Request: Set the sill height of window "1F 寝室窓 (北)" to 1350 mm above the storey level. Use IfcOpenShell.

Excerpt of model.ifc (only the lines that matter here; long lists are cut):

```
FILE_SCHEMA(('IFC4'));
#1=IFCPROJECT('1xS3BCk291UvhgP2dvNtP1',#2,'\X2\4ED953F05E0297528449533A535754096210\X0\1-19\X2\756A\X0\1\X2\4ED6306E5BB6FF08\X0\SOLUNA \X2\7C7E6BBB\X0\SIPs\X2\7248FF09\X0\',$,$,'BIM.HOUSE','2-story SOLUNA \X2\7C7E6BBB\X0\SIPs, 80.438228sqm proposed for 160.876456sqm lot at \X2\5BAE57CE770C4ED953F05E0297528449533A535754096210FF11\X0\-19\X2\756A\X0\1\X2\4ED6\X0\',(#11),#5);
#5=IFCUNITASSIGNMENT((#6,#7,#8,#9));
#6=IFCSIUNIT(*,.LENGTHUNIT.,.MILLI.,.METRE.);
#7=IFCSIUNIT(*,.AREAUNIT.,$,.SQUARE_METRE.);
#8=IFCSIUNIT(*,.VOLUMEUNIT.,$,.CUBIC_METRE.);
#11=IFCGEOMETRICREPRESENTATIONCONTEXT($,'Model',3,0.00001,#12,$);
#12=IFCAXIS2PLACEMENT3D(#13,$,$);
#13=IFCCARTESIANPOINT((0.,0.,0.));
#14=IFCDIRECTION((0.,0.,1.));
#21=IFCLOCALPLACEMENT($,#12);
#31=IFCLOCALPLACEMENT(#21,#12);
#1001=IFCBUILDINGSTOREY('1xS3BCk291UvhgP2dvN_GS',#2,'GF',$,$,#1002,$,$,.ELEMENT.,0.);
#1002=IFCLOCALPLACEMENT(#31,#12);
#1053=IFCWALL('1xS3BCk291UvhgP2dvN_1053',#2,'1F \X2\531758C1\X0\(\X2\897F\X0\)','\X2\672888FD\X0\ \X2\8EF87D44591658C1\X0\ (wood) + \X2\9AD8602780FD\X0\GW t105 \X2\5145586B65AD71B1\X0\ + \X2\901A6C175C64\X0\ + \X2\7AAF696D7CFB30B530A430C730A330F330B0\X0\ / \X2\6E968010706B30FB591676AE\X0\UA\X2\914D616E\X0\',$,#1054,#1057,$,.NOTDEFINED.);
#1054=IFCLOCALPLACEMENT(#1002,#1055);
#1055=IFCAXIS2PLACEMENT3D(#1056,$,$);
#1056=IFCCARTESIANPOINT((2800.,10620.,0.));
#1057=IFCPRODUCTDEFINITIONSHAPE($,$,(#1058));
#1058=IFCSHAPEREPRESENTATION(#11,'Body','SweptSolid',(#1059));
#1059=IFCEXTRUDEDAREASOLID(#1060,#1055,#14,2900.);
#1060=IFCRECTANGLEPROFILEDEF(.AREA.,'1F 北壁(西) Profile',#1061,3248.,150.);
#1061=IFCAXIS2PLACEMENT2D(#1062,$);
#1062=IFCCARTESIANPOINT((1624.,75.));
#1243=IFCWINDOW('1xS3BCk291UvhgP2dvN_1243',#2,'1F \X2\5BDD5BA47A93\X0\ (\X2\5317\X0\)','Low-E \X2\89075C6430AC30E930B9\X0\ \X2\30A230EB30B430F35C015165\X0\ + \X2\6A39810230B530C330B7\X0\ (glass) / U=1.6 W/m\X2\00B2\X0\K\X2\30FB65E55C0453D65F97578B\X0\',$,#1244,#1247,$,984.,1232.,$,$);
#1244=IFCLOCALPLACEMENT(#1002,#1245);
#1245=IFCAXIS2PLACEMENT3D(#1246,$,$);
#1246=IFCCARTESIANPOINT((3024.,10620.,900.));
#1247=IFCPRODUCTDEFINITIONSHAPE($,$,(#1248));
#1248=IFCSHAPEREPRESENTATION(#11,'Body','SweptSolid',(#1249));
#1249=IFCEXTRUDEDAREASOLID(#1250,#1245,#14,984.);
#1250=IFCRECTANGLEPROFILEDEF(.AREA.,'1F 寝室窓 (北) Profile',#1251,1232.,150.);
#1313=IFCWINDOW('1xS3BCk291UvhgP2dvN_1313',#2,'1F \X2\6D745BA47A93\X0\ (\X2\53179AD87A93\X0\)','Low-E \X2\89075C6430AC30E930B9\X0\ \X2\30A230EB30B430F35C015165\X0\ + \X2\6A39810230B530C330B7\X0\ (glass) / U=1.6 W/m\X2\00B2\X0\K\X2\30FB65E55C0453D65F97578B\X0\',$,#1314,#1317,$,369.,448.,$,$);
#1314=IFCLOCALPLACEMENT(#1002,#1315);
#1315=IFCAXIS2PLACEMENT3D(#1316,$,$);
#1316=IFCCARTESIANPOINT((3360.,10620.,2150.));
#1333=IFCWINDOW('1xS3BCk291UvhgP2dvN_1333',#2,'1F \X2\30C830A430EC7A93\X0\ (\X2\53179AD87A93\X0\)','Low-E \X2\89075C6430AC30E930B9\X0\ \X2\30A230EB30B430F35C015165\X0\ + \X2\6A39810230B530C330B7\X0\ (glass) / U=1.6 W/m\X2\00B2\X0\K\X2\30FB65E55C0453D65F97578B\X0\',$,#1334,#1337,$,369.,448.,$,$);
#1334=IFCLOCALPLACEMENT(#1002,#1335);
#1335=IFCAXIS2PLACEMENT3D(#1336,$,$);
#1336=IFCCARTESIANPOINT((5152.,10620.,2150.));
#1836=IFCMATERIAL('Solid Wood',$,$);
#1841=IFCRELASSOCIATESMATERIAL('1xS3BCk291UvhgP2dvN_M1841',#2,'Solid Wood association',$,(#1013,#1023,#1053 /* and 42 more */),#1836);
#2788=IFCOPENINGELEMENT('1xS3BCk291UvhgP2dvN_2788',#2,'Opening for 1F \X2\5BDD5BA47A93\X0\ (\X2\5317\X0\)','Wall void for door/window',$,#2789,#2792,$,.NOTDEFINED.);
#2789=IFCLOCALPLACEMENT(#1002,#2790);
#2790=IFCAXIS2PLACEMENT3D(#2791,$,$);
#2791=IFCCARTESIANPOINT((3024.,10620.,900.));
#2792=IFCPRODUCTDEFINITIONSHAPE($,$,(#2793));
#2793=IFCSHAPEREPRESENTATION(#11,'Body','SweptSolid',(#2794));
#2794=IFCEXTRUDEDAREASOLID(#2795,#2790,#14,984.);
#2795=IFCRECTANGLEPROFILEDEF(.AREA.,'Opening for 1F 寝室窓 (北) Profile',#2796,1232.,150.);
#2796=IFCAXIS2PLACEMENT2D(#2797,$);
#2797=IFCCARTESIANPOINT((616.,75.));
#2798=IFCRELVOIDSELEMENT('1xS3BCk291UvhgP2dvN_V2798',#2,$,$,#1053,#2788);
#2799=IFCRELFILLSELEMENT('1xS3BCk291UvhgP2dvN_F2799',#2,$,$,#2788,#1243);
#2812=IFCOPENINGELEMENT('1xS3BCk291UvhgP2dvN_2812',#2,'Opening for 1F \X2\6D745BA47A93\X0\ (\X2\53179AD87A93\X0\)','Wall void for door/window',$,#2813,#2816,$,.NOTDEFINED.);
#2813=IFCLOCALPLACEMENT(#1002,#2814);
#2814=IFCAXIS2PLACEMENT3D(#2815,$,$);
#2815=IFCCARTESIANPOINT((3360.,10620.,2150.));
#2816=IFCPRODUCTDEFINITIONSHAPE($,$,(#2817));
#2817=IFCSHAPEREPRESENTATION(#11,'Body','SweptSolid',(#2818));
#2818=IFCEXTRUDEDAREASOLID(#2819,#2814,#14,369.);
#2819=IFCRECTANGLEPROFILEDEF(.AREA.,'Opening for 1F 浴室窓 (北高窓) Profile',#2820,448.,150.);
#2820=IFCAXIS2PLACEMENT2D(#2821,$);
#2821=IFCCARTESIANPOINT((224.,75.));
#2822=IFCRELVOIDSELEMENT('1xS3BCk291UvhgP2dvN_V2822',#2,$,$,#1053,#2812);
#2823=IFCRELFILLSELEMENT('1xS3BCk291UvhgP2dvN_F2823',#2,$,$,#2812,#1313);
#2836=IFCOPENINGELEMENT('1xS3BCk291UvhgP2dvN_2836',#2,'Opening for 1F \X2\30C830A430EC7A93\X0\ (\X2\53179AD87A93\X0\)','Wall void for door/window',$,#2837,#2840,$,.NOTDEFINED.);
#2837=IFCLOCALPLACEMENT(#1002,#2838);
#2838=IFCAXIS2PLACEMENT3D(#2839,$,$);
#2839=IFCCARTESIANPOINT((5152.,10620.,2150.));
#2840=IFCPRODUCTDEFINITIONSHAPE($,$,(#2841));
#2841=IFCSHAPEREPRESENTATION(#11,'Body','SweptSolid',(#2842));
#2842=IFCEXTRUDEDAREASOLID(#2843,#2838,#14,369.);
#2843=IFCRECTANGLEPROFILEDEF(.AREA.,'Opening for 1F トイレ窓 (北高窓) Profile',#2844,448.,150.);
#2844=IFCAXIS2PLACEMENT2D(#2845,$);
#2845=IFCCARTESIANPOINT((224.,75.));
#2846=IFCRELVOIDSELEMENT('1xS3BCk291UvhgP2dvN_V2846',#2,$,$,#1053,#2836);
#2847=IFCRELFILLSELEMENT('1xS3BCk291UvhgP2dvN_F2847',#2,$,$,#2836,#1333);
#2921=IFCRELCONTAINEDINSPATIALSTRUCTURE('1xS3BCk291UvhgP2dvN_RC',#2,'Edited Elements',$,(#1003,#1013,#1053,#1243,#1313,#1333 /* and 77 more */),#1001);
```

```python
import numpy as np
import ifcopenshell
import ifcopenshell.api.geometry
import ifcopenshell.geom
import ifcopenshell.util.element
import ifcopenshell.util.placement
import ifcopenshell.util.shape
import ifcopenshell.util.unit

model = ifcopenshell.open("model.ifc")
unit_scale = ifcopenshell.util.unit.calculate_unit_scale(model)

window = model.by_guid("1xS3BCk291UvhgP2dvN_1243")
opening = window.FillsVoids[0].RelatingOpeningElement
storey = ifcopenshell.util.element.get_container(window, ifc_class="IfcBuildingStorey")
level = ifcopenshell.util.placement.get_local_placement(storey.ObjectPlacement)[2, 3]

# The opening's origin need not be at the sill, so measure its lowest point.
shape = ifcopenshell.geom.create_shape(ifcopenshell.geom.settings(), opening)
bottom = ifcopenshell.util.shape.get_shape_bottom_elevation(shape, shape.geometry) / unit_scale
dz = level + 1.35 / unit_scale - bottom

shift = np.array([0.0, 0.0, dz])
# The window is not placed relative to its opening, so move both.
for product in (opening, window):
    matrix = ifcopenshell.util.placement.get_local_placement(product.ObjectPlacement)
    matrix[:3, 3] += shift
    ifcopenshell.api.geometry.edit_object_placement(model, product=product, matrix=matrix, is_si=False)

print(f"moved by {dz * unit_scale:+.3f} m")

model.write("model_rev.ifc")
```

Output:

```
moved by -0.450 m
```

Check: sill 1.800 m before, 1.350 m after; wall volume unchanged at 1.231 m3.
